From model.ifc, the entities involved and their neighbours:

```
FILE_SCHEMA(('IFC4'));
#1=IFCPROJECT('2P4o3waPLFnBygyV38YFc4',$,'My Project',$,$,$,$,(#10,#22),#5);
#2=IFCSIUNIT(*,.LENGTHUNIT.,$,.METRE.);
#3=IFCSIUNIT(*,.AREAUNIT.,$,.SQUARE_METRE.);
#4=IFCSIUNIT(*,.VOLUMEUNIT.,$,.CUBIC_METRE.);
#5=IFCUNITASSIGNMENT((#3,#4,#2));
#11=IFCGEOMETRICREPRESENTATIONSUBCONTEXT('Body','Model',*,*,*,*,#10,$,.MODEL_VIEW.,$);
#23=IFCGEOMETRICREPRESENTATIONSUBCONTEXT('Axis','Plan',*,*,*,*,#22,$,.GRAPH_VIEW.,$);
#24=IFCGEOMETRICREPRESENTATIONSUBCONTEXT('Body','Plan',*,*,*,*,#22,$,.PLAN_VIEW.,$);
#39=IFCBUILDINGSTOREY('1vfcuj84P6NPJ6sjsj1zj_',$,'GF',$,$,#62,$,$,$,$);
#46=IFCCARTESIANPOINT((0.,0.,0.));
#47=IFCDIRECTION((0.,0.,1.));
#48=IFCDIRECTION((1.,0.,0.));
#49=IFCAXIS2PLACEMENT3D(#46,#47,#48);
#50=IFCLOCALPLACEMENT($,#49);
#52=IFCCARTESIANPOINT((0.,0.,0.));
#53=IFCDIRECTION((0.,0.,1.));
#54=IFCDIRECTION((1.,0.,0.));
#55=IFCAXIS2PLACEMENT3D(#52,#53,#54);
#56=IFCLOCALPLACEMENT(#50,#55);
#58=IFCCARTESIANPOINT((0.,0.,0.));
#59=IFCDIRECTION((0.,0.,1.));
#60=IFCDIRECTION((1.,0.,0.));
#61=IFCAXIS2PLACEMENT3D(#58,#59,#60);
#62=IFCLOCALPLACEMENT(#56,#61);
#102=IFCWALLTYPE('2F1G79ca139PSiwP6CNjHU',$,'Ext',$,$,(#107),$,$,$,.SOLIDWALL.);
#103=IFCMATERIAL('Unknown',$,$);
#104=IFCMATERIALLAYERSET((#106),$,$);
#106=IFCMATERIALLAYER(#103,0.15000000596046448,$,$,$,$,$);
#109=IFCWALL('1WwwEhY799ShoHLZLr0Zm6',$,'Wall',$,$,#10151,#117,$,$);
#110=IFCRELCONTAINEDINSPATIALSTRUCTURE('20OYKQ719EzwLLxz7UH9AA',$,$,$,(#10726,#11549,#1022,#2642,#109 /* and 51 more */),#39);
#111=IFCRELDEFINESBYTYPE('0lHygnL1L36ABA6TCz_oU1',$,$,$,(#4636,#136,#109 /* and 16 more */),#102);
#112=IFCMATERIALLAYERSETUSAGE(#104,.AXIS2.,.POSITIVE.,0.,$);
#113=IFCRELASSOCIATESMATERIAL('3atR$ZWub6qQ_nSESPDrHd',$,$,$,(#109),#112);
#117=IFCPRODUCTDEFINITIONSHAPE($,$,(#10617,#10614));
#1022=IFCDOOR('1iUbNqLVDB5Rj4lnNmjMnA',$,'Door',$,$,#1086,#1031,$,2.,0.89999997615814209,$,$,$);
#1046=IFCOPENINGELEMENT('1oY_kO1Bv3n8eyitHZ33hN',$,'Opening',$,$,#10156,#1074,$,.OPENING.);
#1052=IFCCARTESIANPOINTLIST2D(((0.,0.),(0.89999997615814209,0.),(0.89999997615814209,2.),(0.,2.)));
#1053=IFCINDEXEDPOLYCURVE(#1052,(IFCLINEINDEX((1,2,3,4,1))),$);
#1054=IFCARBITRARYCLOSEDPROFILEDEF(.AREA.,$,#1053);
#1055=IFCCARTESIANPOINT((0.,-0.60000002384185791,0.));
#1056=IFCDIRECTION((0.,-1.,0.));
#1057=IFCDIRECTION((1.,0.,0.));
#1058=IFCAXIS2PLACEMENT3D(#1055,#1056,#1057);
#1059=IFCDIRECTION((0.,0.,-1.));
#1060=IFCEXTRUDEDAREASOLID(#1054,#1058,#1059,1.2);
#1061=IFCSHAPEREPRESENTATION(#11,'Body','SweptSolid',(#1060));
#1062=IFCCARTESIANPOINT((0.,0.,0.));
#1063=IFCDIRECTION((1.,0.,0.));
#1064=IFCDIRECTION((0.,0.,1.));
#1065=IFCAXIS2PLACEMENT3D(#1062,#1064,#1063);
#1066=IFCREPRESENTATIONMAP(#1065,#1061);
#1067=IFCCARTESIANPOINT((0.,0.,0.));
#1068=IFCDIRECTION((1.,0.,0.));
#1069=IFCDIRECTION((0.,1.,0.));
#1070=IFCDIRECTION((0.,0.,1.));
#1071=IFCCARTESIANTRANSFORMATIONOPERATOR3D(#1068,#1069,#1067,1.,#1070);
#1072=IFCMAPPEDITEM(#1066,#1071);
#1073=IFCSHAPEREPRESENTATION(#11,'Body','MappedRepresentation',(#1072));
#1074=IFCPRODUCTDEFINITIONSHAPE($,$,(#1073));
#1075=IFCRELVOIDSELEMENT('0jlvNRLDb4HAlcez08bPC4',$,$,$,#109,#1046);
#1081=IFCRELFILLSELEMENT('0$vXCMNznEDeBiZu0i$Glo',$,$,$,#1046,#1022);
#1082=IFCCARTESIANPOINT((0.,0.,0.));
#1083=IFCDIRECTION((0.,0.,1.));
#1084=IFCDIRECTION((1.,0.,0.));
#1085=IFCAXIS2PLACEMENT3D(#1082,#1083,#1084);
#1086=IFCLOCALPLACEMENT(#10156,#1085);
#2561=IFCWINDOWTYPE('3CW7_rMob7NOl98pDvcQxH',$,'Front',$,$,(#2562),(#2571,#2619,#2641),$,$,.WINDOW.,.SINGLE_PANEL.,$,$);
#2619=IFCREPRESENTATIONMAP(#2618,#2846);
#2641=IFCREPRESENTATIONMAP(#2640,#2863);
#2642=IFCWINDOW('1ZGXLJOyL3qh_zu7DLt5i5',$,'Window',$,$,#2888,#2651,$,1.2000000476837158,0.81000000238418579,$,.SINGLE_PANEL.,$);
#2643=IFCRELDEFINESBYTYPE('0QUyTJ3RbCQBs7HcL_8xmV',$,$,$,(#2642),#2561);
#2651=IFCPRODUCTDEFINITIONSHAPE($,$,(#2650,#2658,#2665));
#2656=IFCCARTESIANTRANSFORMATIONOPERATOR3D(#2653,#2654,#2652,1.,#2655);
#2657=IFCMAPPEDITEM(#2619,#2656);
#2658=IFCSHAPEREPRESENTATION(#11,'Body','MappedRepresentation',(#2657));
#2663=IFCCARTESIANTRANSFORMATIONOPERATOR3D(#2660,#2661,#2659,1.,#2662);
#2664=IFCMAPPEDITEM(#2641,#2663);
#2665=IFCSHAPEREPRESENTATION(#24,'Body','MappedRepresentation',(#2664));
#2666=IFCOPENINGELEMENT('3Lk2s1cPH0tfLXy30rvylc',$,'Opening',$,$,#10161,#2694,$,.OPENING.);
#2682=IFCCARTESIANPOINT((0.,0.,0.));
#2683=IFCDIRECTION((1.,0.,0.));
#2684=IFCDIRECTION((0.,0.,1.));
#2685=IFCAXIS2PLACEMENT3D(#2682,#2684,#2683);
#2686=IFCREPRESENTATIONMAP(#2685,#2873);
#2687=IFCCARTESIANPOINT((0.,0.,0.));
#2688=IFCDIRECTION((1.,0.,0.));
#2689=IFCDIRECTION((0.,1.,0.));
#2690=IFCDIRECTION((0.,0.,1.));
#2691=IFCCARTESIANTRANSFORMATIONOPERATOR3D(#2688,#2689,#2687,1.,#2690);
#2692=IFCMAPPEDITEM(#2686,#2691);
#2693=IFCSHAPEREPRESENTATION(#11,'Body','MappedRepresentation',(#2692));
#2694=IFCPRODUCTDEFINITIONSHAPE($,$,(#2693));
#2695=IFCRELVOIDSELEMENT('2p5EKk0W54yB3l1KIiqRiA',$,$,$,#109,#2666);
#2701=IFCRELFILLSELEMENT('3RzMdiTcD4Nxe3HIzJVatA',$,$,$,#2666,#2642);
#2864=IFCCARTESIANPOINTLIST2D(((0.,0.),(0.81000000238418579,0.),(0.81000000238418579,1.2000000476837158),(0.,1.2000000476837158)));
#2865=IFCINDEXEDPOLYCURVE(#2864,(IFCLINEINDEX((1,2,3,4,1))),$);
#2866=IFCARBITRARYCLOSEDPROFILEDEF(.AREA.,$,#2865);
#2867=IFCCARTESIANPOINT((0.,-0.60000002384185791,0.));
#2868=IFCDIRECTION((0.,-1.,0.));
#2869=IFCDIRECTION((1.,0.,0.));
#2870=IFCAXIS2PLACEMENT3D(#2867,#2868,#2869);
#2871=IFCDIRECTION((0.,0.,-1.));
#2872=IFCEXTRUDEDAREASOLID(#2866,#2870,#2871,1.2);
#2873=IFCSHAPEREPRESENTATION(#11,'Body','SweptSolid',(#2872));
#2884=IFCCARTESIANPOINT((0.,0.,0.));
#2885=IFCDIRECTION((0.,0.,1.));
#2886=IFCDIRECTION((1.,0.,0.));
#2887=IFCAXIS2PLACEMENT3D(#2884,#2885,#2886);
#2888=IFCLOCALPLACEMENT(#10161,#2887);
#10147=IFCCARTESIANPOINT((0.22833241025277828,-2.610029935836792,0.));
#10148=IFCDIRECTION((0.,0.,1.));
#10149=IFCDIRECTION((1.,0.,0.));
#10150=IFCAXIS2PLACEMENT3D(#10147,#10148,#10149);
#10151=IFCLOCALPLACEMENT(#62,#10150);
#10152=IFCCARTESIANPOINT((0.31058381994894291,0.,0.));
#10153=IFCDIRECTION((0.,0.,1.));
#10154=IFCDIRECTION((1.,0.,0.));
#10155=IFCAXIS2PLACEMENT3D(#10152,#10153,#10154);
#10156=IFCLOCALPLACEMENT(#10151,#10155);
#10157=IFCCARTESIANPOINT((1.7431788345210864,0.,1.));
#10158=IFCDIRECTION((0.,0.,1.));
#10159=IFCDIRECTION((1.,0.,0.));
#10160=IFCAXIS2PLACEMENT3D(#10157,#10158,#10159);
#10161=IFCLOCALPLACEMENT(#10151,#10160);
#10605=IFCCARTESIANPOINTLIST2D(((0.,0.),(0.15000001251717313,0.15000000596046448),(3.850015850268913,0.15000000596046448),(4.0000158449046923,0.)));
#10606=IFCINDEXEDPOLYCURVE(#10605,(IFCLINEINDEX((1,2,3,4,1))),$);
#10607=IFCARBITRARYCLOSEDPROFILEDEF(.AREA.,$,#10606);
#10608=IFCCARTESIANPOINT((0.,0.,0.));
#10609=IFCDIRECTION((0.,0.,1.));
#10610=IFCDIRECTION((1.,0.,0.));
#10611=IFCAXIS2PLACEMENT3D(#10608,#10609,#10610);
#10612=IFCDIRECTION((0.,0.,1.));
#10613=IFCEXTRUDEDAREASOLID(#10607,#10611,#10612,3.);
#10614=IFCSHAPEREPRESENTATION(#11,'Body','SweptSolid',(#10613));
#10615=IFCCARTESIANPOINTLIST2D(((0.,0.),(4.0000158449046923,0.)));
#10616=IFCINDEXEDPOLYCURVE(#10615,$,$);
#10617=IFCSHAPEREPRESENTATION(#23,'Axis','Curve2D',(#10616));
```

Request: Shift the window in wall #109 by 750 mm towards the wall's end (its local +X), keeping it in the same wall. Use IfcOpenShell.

```python
import ifcopenshell
import ifcopenshell.api.geometry
import ifcopenshell.util.placement

model = ifcopenshell.open("model.ifc")

window = model.by_guid("1ZGXLJOyL3qh_zu7DLt5i5")
opening = window.FillsVoids[0].RelatingOpeningElement
wall = opening.VoidsElements[0].RelatingBuildingElement

wall_matrix = ifcopenshell.util.placement.get_local_placement(wall.ObjectPlacement)
shift = wall_matrix[:3, 0] * 0.75
before = ifcopenshell.util.placement.get_local_placement(window.ObjectPlacement)[:3, 3].copy()

# The window is placed relative to its opening, so it follows when the opening moves.
matrix = ifcopenshell.util.placement.get_local_placement(opening.ObjectPlacement)
matrix[:3, 3] += shift
ifcopenshell.api.geometry.edit_object_placement(
    model, product=opening, matrix=matrix, is_si=False, should_transform_children=True
)

after = ifcopenshell.util.placement.get_local_placement(window.ObjectPlacement)[:3, 3]
print("window moved by", (after - before).round(3) + 0.0)

model.write("model_v2.ifc")
```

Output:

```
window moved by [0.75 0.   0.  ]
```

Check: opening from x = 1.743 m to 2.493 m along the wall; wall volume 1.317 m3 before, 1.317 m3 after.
